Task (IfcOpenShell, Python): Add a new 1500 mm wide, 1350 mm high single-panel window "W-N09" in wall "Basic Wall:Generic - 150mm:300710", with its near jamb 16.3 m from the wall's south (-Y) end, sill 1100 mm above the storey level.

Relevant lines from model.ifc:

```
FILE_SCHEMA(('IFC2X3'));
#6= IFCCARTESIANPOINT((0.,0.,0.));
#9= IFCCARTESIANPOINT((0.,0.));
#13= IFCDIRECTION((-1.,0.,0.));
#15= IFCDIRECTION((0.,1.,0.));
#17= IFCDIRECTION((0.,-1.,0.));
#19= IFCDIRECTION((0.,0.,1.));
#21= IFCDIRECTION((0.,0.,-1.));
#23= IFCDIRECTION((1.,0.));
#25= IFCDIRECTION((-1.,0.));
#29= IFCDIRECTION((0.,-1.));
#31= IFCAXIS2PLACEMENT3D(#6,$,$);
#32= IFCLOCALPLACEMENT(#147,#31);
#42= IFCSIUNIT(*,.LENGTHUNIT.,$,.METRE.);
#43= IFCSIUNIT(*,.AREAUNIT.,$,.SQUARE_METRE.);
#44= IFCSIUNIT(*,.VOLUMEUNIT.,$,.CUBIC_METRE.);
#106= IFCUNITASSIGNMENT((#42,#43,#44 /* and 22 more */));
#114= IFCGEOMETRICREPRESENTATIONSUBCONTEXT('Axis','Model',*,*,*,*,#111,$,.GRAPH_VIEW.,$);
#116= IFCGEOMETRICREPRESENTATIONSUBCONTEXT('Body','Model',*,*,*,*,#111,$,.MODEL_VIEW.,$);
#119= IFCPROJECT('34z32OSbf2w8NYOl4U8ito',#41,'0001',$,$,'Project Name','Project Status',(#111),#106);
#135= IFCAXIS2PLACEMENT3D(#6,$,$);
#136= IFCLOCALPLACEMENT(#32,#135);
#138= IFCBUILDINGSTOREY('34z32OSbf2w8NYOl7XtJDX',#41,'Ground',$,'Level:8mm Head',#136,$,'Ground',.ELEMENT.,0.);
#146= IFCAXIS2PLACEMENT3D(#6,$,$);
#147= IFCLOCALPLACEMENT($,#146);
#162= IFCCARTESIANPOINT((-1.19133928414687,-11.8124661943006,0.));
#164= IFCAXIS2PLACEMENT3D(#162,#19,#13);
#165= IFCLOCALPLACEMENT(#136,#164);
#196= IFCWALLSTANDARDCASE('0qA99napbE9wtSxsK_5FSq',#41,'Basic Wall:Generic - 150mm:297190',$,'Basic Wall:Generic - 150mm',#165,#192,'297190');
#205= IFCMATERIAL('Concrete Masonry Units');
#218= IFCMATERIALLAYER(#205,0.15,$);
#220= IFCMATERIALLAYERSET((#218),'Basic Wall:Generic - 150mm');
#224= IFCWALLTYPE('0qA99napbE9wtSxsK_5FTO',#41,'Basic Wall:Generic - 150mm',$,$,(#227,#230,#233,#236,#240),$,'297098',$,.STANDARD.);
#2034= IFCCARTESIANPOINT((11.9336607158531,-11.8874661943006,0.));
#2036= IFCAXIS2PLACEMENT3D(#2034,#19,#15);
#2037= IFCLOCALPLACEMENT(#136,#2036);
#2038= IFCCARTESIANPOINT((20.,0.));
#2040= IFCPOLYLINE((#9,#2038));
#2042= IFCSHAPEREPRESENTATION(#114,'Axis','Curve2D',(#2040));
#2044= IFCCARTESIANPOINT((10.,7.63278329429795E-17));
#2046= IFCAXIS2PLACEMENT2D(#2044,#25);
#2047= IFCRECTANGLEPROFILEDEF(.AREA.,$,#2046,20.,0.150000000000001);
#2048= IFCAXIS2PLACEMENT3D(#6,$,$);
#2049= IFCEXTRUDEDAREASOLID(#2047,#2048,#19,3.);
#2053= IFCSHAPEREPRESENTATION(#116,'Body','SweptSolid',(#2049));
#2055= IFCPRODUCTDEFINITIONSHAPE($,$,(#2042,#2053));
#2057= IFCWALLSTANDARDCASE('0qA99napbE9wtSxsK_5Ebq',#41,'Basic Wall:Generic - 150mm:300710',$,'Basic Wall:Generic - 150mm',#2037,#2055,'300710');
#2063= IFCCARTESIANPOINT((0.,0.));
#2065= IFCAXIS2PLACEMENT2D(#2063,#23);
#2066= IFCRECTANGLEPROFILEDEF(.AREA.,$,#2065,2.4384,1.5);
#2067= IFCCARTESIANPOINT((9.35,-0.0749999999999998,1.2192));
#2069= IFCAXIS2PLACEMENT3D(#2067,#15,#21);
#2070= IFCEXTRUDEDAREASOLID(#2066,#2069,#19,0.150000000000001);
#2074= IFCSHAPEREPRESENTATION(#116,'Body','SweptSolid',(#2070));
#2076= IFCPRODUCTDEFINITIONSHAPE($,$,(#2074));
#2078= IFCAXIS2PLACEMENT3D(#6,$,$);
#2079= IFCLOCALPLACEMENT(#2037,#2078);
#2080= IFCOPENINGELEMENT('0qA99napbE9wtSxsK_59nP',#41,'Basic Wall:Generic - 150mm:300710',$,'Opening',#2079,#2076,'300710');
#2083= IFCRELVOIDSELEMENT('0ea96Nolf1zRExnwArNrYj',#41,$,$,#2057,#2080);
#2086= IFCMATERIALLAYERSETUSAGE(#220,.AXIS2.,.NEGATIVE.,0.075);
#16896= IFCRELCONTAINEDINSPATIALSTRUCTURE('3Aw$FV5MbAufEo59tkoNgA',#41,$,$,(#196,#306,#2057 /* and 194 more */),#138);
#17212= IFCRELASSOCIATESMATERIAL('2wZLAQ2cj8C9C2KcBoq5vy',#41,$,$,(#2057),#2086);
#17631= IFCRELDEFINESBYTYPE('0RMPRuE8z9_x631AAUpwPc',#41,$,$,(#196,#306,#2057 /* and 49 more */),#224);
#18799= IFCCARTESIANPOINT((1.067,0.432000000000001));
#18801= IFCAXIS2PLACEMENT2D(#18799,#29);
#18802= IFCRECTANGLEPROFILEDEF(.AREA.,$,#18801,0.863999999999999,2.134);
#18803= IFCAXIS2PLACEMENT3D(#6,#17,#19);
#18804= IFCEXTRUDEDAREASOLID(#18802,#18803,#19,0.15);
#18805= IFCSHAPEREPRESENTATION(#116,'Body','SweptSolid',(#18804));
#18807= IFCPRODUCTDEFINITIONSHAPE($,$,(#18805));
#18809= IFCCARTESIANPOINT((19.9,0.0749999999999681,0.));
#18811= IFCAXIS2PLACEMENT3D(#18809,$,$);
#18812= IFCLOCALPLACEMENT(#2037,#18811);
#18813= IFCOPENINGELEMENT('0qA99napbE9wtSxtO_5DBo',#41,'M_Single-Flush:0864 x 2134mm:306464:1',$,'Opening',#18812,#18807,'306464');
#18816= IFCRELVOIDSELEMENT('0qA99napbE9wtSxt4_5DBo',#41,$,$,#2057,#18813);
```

```python
import numpy as np
import ifcopenshell
import ifcopenshell.api.feature
import ifcopenshell.api.geometry
import ifcopenshell.api.root
import ifcopenshell.api.spatial
import ifcopenshell.api.type
import ifcopenshell.geom
import ifcopenshell.util.element
import ifcopenshell.util.placement
import ifcopenshell.util.representation
import ifcopenshell.util.shape
import ifcopenshell.util.unit

model = ifcopenshell.open("model.ifc")
unit_scale = ifcopenshell.util.unit.calculate_unit_scale(model)
settings = ifcopenshell.geom.settings()


def volume(element):
    """Net volume in cubic metres, openings subtracted."""
    shape = ifcopenshell.geom.create_shape(settings, element)
    return ifcopenshell.util.shape.get_volume(shape.geometry)


wall = model.by_id(2057)
storey = ifcopenshell.util.element.get_container(wall, ifc_class="IfcBuildingStorey")
context = ifcopenshell.util.representation.get_context(model, "Model", "Body", "MODEL_VIEW")
before = volume(wall)

width, height, from_end, sill = 1.5, 1.35, 16.3, 1.1  # metres

# The wall runs along its own X axis, and the end named is its -X end.
wall_shape = ifcopenshell.geom.create_shape(settings, wall)
x, y, z = ifcopenshell.util.shape.get_vertices(wall_shape.geometry).T
start = x.min() + from_end
face, thickness = float(y.min()), float(y.max() - y.min())
wall_matrix = ifcopenshell.util.placement.get_local_placement(wall.ObjectPlacement)
level = ifcopenshell.util.placement.get_local_placement(storey.ObjectPlacement)[2, 3]


def in_wall(x, y):
    """Placement at x, y metres in the wall's axes, at sill height."""
    matrix = wall_matrix.copy()
    matrix[:, 3] = wall_matrix @ np.array([x / unit_scale, y / unit_scale, 0.0, 1.0])
    matrix[2, 3] = level + sill / unit_scale
    return matrix


# Opening: a box that overshoots both wall faces by 50 mm.
opening = ifcopenshell.api.root.create_entity(model, ifc_class="IfcOpeningElement")
box = ifcopenshell.api.geometry.add_wall_representation(
    model, context=context, length=width, height=height, thickness=thickness + 0.1
)
ifcopenshell.api.geometry.assign_representation(model, product=opening, representation=box)
ifcopenshell.api.geometry.edit_object_placement(model, product=opening, matrix=in_wall(start, face - 0.05), is_si=False)
ifcopenshell.api.feature.add_feature(model, feature=opening, element=wall)

window = ifcopenshell.api.root.create_entity(model, ifc_class="IfcWindow", name="W-N09")
window.OverallWidth, window.OverallHeight = width / unit_scale, height / unit_scale
body = ifcopenshell.api.geometry.add_window_representation(
    model,
    context=context,
    overall_width=window.OverallWidth,
    overall_height=window.OverallHeight,
    partition_type="SINGLE_PANEL",
)
ifcopenshell.api.geometry.assign_representation(model, product=window, representation=body)
ifcopenshell.api.spatial.assign_container(model, products=[window], relating_structure=storey)
fills = ifcopenshell.api.feature.add_filling(model, opening=opening, element=window)
fills.OwnerHistory = window.OwnerHistory  # required in IFC2X3

# IFC2X3 keeps the operation on the window style.
style = ifcopenshell.api.root.create_entity(model, ifc_class="IfcWindowStyle", name="W-N09")
style.OperationType, style.ConstructionType = "SINGLE_PANEL", "NOTDEFINED"
style.ParameterTakesPrecedence = style.Sizeable = False
ifcopenshell.api.type.assign_type(model, related_objects=[window], relating_type=style)

# Centre the window in the wall's thickness.
ifcopenshell.api.geometry.edit_object_placement(model, product=window, matrix=in_wall(start, face), is_si=False)
window_shape = ifcopenshell.geom.create_shape(settings, window)
depth = ifcopenshell.util.shape.get_vertices(window_shape.geometry)[:, 1]
offset = face + thickness / 2 - (depth.min() + depth.max()) / 2
ifcopenshell.api.geometry.edit_object_placement(model, product=window, matrix=in_wall(start, offset), is_si=False)

after = volume(wall)

print(f"wall volume {before:.3f} -> {after:.3f} m3")

model.write("model_rev.ifc")
```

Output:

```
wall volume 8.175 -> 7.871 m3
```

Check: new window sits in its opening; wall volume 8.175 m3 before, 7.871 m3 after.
